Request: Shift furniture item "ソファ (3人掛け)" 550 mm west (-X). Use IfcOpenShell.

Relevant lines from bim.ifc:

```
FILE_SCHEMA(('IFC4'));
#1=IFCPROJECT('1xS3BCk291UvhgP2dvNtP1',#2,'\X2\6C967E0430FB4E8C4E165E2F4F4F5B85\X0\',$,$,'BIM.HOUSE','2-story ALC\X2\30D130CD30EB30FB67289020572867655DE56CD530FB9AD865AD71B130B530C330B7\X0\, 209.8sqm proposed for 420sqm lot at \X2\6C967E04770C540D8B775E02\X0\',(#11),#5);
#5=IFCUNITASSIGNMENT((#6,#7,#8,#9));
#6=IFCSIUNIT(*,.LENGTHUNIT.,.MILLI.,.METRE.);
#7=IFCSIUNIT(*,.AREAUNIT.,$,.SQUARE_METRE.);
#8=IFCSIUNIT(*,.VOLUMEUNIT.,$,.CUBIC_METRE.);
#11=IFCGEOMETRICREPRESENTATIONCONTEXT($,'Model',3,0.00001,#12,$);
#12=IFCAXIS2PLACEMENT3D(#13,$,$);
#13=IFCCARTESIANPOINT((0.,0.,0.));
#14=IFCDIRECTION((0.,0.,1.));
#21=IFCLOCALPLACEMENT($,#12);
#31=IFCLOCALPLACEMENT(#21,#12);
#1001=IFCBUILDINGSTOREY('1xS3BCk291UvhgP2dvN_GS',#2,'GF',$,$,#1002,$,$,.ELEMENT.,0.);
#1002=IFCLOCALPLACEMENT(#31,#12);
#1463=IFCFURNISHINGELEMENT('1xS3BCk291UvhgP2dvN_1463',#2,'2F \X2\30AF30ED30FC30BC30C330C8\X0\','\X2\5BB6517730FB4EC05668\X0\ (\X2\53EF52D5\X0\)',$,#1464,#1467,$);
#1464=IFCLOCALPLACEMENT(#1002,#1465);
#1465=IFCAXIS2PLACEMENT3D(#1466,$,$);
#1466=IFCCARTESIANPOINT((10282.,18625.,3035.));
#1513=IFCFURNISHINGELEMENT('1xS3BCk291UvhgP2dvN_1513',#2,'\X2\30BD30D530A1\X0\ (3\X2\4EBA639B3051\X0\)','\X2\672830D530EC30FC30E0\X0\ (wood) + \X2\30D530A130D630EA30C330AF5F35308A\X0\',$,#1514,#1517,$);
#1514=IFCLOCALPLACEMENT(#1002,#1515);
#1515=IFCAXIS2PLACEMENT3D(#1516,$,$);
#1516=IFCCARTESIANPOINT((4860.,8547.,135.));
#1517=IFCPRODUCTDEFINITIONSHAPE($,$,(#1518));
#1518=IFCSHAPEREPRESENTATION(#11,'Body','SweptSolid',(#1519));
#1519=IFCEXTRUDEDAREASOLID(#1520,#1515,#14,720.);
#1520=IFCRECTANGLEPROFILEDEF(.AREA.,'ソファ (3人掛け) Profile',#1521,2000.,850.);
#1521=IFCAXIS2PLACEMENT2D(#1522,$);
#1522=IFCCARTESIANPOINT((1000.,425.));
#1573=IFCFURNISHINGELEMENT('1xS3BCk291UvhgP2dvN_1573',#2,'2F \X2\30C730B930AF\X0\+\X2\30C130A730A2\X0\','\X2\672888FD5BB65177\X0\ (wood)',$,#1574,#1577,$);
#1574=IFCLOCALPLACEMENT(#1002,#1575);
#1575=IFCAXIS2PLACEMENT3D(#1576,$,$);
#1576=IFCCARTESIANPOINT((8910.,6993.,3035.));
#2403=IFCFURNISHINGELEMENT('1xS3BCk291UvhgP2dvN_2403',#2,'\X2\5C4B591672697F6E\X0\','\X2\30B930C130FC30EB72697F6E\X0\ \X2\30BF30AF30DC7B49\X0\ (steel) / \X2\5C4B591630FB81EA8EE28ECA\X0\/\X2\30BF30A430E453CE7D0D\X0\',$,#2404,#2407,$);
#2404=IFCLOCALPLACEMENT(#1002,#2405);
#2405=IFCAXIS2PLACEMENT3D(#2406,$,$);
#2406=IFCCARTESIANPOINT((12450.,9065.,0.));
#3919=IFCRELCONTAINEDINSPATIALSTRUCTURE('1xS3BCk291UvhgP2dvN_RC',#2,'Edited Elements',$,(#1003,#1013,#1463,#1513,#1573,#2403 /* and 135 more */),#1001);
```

```python
import ifcopenshell
import ifcopenshell.api.geometry
import ifcopenshell.util.placement

model = ifcopenshell.open("bim.ifc")

item = model.by_guid("1xS3BCk291UvhgP2dvN_1513")
matrix = ifcopenshell.util.placement.get_local_placement(item.ObjectPlacement)
matrix[0, 3] -= 550.0
ifcopenshell.api.geometry.edit_object_placement(model, product=item, matrix=matrix, is_si=False)

print(ifcopenshell.util.placement.get_local_placement(item.ObjectPlacement).round(3) + 0.0)

model.write("bim_updated.ifc")
```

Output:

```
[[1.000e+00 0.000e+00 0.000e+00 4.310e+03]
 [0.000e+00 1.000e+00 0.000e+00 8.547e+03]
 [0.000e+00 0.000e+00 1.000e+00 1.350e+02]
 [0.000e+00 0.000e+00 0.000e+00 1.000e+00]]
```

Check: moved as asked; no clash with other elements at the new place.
